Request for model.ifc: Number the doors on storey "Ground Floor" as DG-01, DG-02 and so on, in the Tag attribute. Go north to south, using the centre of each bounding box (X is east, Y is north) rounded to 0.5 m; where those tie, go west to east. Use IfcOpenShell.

First a look at what the model holds.

```python
import ifcopenshell
import ifcopenshell.util.element
import ifcopenshell.util.placement

model = ifcopenshell.open("model.ifc")
print(model.schema)
storey = next(s for s in model.by_type("IfcBuildingStorey") if s.Name == "Ground Floor")
doors = [e for e in ifcopenshell.util.element.get_decomposition(storey) if e.is_a("IfcDoor")]
for e in sorted(doors, key=lambda e: e.id()):
    origin = ifcopenshell.util.placement.get_local_placement(e.ObjectPlacement)[:3, 3]
    print(e.id(), e.Tag, e.Name, origin.round(2) + 0.0, sep=" | ")
```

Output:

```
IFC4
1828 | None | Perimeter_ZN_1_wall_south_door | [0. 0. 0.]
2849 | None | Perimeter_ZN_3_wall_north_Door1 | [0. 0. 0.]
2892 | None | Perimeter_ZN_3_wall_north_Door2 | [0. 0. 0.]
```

```python
import ifcopenshell
import ifcopenshell.geom
import ifcopenshell.util.element
import ifcopenshell.util.shape

model = ifcopenshell.open("model.ifc")
settings = ifcopenshell.geom.settings()
settings.set("use-world-coords", True)


def centre(element):
    shape = ifcopenshell.geom.create_shape(settings, element)
    return ifcopenshell.util.shape.get_bbox_centroid(shape.geometry)


storey = next(s for s in model.by_type("IfcBuildingStorey") if s.Name == "Ground Floor")
doors = [e for e in ifcopenshell.util.element.get_decomposition(storey) if e.is_a("IfcDoor")]

# Insertion points can sit at a corner or the storey origin, so sort by the geometry (in metres).
centres = {e: centre(e) for e in doors}
doors.sort(key=lambda e: (-round(centres[e][1] / 0.5), centres[e][0]))

for i, e in enumerate(doors, start=1):
    number = f"DG-{i:02d}"
    e.Tag = number
    print(e.id(), number)

model.write("model_rev.ifc")
```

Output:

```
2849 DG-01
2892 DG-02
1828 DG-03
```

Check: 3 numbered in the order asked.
